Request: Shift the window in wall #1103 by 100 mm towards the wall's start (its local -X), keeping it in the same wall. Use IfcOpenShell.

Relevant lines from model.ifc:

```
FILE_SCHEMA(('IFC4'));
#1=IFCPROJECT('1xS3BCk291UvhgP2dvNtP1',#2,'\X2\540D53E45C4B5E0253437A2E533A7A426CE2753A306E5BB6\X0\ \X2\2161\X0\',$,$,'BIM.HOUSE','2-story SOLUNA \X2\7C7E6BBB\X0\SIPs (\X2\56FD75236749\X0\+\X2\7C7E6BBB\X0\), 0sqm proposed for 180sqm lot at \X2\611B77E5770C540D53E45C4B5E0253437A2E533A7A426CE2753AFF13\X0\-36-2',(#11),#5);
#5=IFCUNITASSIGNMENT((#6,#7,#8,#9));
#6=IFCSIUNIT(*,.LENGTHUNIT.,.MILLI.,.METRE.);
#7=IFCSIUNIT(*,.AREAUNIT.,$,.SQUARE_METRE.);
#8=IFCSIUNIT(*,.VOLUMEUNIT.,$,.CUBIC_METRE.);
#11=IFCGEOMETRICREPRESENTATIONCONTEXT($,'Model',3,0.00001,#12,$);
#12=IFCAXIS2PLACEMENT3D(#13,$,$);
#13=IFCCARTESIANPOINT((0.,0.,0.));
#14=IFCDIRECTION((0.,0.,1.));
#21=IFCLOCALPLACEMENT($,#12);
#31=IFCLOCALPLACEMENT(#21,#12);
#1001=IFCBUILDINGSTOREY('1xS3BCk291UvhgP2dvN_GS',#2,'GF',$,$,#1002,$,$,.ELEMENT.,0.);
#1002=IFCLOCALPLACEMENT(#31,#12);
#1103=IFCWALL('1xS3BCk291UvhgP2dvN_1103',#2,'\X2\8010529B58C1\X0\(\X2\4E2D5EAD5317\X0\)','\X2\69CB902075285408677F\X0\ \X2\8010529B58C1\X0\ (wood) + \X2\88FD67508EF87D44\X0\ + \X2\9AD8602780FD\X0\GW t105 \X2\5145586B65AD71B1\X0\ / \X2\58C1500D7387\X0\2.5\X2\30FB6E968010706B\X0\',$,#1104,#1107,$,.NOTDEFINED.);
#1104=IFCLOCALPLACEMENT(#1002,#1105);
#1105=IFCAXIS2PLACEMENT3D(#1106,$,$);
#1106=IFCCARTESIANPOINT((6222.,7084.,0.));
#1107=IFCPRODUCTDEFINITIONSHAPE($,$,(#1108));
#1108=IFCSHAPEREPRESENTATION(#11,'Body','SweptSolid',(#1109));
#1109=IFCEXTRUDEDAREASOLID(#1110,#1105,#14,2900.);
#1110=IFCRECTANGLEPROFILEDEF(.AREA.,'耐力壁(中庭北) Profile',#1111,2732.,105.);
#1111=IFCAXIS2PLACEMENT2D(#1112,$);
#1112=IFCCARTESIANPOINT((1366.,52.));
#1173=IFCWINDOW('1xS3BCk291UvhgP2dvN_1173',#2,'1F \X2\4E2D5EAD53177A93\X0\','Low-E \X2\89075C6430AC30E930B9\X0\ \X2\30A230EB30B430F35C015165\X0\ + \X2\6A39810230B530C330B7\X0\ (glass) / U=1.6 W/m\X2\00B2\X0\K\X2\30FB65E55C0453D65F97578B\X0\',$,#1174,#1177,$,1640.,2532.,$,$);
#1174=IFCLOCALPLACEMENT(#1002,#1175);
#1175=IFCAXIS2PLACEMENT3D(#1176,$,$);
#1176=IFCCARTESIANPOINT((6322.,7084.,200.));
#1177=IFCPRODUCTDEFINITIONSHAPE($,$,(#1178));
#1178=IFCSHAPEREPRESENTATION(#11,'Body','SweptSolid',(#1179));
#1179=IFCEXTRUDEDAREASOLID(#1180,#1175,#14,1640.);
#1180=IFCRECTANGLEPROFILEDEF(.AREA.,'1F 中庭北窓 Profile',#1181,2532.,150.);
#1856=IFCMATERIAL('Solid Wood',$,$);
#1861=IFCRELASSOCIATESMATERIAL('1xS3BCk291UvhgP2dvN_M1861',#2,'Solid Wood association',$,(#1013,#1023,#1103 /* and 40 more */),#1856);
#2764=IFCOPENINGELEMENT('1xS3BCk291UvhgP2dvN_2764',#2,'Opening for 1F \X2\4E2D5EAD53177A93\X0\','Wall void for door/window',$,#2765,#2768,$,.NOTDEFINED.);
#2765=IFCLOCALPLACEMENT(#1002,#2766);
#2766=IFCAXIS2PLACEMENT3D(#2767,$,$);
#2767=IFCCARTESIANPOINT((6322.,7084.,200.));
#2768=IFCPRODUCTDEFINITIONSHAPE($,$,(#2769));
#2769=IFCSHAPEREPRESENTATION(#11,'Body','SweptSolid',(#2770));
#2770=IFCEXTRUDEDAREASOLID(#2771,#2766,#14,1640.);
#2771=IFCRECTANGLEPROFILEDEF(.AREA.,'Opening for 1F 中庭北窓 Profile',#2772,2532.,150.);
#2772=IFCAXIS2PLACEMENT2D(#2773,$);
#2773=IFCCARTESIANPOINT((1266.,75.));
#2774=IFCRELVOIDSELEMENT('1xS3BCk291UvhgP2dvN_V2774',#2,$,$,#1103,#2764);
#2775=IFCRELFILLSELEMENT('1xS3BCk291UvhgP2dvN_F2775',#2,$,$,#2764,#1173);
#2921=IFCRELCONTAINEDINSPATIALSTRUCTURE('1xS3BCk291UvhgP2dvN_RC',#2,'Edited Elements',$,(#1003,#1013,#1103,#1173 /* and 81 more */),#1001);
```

```python
import ifcopenshell
import ifcopenshell.api.geometry
import ifcopenshell.util.placement
import ifcopenshell.util.unit

model = ifcopenshell.open("model.ifc")
unit_scale = ifcopenshell.util.unit.calculate_unit_scale(model)

window = model.by_guid("1xS3BCk291UvhgP2dvN_1173")
opening = window.FillsVoids[0].RelatingOpeningElement
wall = opening.VoidsElements[0].RelatingBuildingElement

wall_matrix = ifcopenshell.util.placement.get_local_placement(wall.ObjectPlacement)
shift = wall_matrix[:3, 0] * -0.1 / unit_scale
before = ifcopenshell.util.placement.get_local_placement(window.ObjectPlacement)[:3, 3].copy()

# The window is not placed relative to its opening, so move both.
for product in (opening, window):
    matrix = ifcopenshell.util.placement.get_local_placement(product.ObjectPlacement)
    matrix[:3, 3] += shift
    ifcopenshell.api.geometry.edit_object_placement(model, product=product, matrix=matrix, is_si=False)

after = ifcopenshell.util.placement.get_local_placement(window.ObjectPlacement)[:3, 3]
print("window moved by", (after - before).round(3) + 0.0)

model.write("model_rev.ifc")
```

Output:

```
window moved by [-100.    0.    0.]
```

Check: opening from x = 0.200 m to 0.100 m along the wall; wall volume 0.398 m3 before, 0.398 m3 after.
